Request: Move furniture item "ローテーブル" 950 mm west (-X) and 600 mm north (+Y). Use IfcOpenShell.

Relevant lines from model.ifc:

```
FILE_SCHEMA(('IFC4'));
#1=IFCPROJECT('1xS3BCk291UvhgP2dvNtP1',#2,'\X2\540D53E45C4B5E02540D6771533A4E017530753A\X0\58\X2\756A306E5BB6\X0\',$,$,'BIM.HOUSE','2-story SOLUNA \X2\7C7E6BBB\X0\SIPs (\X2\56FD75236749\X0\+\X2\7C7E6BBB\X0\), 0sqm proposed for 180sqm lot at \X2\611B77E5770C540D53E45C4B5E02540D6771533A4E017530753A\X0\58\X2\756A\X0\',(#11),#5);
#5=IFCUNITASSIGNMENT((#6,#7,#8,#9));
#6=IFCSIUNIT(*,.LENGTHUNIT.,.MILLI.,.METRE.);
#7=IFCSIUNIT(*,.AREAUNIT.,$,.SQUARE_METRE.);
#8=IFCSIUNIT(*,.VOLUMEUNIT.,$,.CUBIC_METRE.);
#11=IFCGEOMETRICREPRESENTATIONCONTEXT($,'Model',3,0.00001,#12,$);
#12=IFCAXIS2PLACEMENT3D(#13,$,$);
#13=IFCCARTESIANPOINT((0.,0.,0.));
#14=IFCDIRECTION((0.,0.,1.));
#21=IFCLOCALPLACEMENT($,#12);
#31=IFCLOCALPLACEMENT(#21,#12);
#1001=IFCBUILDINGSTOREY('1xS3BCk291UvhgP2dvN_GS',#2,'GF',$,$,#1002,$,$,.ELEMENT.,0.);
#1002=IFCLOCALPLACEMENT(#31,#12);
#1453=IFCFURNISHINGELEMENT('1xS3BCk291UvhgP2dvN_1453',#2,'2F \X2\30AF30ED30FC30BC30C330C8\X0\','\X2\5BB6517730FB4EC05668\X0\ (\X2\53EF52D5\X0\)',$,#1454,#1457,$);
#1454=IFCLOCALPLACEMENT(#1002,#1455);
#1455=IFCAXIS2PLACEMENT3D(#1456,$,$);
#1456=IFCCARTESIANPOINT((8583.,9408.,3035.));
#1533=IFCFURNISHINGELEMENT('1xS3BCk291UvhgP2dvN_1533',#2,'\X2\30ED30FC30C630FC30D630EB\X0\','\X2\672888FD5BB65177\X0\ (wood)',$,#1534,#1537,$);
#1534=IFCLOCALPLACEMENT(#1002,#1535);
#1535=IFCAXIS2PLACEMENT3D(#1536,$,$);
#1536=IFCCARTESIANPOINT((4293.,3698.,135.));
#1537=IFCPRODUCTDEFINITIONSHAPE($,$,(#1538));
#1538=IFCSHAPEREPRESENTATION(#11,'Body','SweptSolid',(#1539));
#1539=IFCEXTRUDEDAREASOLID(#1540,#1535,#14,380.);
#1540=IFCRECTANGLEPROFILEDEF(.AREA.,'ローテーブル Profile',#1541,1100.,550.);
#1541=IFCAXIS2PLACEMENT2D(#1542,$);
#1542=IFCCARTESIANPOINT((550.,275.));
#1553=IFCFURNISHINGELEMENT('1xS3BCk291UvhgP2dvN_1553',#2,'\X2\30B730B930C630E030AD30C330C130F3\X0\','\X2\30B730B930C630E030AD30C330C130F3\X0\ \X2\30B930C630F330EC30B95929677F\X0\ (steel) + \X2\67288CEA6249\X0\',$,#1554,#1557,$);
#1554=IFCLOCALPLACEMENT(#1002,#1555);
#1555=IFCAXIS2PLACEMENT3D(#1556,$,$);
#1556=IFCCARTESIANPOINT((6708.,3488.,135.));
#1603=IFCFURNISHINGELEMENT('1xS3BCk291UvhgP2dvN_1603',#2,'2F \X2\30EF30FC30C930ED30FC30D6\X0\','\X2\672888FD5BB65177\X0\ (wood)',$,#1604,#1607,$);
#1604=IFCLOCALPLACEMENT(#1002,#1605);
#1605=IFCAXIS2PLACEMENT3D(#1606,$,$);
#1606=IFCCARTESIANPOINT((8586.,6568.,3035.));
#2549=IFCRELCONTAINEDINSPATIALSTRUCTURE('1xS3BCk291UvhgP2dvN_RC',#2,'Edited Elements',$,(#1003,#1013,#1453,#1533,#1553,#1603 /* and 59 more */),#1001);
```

```python
import ifcopenshell
import ifcopenshell.api.geometry
import ifcopenshell.util.placement
import ifcopenshell.util.unit

model = ifcopenshell.open("model.ifc")
unit_scale = ifcopenshell.util.unit.calculate_unit_scale(model)

item = model.by_guid("1xS3BCk291UvhgP2dvN_1533")
matrix = ifcopenshell.util.placement.get_local_placement(item.ObjectPlacement)
matrix[0, 3] -= 0.95 / unit_scale
matrix[1, 3] += 0.6 / unit_scale
ifcopenshell.api.geometry.edit_object_placement(model, product=item, matrix=matrix, is_si=False)

print(ifcopenshell.util.placement.get_local_placement(item.ObjectPlacement).round(3) + 0.0)

model.write("model-out.ifc")
```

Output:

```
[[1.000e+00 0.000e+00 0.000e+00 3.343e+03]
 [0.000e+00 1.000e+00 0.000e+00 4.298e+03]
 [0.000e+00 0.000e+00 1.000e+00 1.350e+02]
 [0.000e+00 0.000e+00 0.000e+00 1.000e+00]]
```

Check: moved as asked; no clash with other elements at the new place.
